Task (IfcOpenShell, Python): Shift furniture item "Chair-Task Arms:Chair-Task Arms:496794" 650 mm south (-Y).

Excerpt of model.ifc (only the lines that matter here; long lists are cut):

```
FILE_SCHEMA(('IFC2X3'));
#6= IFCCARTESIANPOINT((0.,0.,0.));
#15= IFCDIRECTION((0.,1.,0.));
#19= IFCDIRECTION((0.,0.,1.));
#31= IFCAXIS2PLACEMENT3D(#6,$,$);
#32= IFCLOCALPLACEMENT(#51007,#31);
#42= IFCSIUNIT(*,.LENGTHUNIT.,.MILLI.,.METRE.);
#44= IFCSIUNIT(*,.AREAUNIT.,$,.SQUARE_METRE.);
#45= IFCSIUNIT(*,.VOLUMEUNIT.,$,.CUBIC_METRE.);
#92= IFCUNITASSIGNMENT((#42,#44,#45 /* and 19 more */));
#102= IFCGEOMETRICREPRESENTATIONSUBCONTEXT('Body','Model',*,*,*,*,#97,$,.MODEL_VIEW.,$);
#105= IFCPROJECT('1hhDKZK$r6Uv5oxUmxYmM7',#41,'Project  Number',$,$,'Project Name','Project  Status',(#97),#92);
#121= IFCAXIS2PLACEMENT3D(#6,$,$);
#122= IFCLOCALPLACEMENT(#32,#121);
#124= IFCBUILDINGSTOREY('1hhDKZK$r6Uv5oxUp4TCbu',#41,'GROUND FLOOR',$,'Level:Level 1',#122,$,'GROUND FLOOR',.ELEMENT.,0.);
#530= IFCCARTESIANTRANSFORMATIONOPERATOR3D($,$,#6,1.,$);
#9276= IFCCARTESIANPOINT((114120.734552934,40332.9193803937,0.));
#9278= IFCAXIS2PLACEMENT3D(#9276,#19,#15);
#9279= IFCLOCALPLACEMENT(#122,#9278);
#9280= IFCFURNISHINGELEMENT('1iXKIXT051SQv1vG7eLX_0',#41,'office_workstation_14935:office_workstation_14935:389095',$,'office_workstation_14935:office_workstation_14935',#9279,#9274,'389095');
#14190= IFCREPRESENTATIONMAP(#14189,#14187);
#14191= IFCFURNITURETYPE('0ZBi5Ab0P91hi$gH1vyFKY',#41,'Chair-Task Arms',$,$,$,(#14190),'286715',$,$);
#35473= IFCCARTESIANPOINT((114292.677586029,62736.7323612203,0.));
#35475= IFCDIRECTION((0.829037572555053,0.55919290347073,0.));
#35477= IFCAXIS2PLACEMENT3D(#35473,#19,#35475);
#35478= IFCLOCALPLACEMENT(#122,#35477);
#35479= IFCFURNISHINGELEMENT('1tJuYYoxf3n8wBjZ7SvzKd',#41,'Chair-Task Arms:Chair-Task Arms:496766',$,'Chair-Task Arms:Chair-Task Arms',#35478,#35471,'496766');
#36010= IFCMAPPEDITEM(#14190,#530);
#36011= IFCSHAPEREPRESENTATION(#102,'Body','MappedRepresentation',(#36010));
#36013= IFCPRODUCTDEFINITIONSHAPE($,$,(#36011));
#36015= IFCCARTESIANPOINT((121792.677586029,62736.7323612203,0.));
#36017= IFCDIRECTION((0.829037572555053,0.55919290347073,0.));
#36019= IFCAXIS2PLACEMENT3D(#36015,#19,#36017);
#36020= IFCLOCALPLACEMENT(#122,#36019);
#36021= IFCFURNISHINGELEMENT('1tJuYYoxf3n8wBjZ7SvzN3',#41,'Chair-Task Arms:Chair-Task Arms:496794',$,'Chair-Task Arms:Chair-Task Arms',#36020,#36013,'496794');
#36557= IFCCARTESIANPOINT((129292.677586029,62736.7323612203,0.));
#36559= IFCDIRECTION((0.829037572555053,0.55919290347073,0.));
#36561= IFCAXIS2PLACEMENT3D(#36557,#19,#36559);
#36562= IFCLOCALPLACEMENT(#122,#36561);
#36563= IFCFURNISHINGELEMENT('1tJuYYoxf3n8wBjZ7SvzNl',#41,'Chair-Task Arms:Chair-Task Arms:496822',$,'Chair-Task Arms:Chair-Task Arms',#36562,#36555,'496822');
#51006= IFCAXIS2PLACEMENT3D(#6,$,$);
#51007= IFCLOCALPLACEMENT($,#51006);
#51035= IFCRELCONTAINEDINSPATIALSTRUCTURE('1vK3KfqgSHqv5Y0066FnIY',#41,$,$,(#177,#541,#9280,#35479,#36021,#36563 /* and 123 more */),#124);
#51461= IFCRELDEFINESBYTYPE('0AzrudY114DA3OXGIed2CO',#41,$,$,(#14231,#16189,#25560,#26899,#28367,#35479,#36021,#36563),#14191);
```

```python
import ifcopenshell
import ifcopenshell.api.geometry
import ifcopenshell.util.placement

model = ifcopenshell.open("model.ifc")

item = model.by_guid("1tJuYYoxf3n8wBjZ7SvzN3")
matrix = ifcopenshell.util.placement.get_local_placement(item.ObjectPlacement)
matrix[1, 3] -= 650.0
ifcopenshell.api.geometry.edit_object_placement(model, product=item, matrix=matrix, is_si=False)

print(ifcopenshell.util.placement.get_local_placement(item.ObjectPlacement).round(3) + 0.0)

model.write("model_rev.ifc")
```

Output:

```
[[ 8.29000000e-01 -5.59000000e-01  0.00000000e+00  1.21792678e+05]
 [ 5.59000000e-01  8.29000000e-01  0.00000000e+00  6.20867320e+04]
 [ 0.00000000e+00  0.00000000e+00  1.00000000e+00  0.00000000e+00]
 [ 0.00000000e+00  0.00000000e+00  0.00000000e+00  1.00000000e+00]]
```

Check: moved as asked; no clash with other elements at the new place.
